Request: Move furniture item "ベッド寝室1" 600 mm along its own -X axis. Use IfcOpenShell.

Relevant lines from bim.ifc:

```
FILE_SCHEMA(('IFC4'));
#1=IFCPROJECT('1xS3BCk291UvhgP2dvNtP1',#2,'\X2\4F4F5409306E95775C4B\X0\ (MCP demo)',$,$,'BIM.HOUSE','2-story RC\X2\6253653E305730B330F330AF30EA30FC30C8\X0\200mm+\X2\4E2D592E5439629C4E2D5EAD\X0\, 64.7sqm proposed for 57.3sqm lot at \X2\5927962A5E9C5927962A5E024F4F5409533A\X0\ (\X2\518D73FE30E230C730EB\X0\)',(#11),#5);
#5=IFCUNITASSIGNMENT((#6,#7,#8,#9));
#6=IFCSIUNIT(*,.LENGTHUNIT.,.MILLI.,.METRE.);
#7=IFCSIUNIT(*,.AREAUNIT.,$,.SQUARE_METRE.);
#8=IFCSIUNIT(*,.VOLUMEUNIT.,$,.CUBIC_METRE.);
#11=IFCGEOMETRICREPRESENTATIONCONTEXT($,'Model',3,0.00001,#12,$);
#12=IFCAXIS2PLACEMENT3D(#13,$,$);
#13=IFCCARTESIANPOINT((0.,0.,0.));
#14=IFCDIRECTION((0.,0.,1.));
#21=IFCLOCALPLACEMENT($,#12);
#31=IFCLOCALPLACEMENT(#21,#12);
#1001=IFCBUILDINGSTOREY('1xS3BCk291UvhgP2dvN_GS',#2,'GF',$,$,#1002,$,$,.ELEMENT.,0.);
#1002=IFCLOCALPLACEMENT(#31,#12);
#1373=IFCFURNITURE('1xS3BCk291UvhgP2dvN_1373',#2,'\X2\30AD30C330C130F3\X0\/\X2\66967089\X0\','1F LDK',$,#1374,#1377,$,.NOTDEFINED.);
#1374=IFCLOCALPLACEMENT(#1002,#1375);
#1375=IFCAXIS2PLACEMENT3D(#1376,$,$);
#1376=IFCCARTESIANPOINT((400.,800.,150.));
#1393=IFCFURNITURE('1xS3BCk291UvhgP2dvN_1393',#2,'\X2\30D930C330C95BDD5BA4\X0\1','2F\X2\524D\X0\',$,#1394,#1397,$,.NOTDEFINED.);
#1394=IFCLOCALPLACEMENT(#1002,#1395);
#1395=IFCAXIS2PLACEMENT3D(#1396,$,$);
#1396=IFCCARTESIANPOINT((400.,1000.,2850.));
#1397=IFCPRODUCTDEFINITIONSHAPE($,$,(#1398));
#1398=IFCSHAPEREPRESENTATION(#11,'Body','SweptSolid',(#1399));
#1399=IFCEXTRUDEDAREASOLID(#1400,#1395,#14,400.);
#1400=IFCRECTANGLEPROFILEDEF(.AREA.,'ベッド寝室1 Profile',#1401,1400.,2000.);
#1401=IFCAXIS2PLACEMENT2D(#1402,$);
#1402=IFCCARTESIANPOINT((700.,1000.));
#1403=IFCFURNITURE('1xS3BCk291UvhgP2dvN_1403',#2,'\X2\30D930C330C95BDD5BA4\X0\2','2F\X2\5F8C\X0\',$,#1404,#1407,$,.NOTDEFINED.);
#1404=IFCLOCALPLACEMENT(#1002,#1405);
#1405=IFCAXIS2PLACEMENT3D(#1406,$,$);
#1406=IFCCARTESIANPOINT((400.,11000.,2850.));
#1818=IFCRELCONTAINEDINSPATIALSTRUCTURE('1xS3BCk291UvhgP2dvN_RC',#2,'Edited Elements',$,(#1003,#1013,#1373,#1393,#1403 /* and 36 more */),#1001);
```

```python
import ifcopenshell
import ifcopenshell.api.geometry
import ifcopenshell.util.placement
import ifcopenshell.util.unit

model = ifcopenshell.open("bim.ifc")
unit_scale = ifcopenshell.util.unit.calculate_unit_scale(model)

item = model.by_guid("1xS3BCk291UvhgP2dvN_1393")
matrix = ifcopenshell.util.placement.get_local_placement(item.ObjectPlacement)
matrix[:3, 3] -= matrix[:3, 0] * 0.6 / unit_scale
ifcopenshell.api.geometry.edit_object_placement(model, product=item, matrix=matrix, is_si=False)

print(ifcopenshell.util.placement.get_local_placement(item.ObjectPlacement).round(3) + 0.0)

model.write("bim-out.ifc")
```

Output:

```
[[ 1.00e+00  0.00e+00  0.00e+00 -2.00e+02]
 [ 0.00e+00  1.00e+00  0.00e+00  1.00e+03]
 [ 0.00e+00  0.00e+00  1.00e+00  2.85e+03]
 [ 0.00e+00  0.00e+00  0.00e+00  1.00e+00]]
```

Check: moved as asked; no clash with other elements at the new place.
